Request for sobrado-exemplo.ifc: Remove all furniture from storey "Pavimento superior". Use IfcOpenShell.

First a look at what the model holds.

```python
import ifcopenshell
import ifcopenshell.util.element

model = ifcopenshell.open("sobrado-exemplo.ifc")
print(model.schema)
storey = next(s for s in model.by_type("IfcBuildingStorey") if s.Name == "Pavimento superior")
furniture = [e for e in ifcopenshell.util.element.get_decomposition(storey) if e.is_a("IfcFurnishingElement")]
seen = {}
for e in furniture:
    element_type = ifcopenshell.util.element.get_type(e)
    name = element_type.Name if element_type not in (None, e) else None
    seen[name] = seen.get(name, 0) + 1
for name, count in sorted(seen.items(), key=str):
    print(count, "x", name)
```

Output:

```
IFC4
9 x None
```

```python
import ifcopenshell
import ifcopenshell.api.root
import ifcopenshell.util.element

model = ifcopenshell.open("sobrado-exemplo.ifc")

storey = next(s for s in model.by_type("IfcBuildingStorey") if s.Name == "Pavimento superior")
furniture = [e for e in ifcopenshell.util.element.get_decomposition(storey) if e.is_a("IfcFurnishingElement")]

for e in furniture:
    ifcopenshell.api.root.remove_product(model, product=e)
print(len(furniture), "removed")

model.write("sobrado-exemplo_rev.ifc")
```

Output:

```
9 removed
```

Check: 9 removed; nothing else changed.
